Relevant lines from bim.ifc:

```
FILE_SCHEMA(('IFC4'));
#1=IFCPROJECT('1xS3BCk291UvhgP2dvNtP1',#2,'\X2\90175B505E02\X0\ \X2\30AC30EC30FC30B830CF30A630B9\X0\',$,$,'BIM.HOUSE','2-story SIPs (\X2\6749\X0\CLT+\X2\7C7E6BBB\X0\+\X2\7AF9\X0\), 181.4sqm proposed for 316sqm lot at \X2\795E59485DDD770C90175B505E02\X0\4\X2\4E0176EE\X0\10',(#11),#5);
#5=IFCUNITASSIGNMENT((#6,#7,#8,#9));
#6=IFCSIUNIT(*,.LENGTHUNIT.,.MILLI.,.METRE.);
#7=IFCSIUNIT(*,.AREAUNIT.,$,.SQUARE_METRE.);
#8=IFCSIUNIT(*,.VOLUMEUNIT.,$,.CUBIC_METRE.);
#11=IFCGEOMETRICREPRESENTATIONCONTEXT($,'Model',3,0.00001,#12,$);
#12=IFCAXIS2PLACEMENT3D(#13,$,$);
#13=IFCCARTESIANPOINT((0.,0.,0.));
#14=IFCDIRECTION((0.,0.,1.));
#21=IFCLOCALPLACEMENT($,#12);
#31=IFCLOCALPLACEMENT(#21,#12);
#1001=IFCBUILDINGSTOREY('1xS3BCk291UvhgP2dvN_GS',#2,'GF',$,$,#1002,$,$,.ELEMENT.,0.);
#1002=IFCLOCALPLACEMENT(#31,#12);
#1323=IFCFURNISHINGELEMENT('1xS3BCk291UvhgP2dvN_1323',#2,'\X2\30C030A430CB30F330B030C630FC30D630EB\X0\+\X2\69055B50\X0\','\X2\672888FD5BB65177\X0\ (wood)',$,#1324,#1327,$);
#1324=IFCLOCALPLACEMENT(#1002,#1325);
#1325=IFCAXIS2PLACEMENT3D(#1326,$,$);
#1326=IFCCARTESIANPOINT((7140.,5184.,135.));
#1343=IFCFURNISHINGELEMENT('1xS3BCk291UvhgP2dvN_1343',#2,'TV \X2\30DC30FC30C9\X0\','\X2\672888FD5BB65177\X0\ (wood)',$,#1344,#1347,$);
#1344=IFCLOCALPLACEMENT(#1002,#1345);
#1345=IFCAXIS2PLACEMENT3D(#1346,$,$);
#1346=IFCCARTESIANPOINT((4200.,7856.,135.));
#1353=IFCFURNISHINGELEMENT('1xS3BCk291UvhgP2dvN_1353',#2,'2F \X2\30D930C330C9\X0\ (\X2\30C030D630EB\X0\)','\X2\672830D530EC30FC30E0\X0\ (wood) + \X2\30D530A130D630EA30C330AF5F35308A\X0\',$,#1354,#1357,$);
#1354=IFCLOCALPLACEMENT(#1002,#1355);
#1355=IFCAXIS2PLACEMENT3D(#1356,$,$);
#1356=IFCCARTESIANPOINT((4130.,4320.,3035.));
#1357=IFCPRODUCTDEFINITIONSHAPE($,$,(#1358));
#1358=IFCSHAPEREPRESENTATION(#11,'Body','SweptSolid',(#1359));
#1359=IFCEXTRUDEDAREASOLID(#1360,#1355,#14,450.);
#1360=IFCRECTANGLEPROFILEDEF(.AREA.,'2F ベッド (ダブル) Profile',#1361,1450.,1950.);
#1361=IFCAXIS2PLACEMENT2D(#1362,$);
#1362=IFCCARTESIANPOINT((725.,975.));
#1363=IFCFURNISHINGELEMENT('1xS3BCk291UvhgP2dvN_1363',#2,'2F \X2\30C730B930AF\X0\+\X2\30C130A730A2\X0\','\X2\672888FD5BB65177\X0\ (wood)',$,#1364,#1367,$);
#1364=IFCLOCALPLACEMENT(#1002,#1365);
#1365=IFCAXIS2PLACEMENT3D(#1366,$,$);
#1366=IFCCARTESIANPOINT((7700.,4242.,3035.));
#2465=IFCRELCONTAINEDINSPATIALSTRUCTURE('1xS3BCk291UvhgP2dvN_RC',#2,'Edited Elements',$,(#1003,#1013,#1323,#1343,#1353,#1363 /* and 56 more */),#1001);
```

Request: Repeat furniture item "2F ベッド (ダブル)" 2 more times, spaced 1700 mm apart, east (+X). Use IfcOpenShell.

```python
import numpy as np
import ifcopenshell
import ifcopenshell.api.geometry
import ifcopenshell.api.root
import ifcopenshell.util.element
import ifcopenshell.util.placement
import ifcopenshell.util.unit

model = ifcopenshell.open("bim.ifc")
unit_scale = ifcopenshell.util.unit.calculate_unit_scale(model)


def reuse_history(source, copy):
    """copy_class also copies each property set's owner history, people and application; keep the originals."""
    for rel in copy.IsDefinedBy:
        if rel.is_a("IfcRelDefinesByProperties") and (history := rel.RelatingPropertyDefinition.OwnerHistory):
            rel.RelatingPropertyDefinition.OwnerHistory = source.OwnerHistory
            ifcopenshell.util.element.remove_deep2(model, history)


source = model.by_guid("1xS3BCk291UvhgP2dvN_1353")
base = ifcopenshell.util.placement.get_local_placement(source.ObjectPlacement)
step = np.array([1.0, 0.0, 0.0]) * 1.7 / unit_scale

for i in range(1, 3):
    copy = ifcopenshell.api.root.copy_class(model, product=source)
    copy.Representation = ifcopenshell.util.element.copy_deep(
        model, source.Representation, exclude=["IfcGeometricRepresentationContext", "IfcRepresentationMap"]
    )
    reuse_history(source, copy)
    matrix = base.copy()
    matrix[:3, 3] += i * step
    print("added at", matrix[:3, 3].round(3) + 0.0)
    ifcopenshell.api.geometry.edit_object_placement(model, product=copy, matrix=matrix, is_si=False)

model.write("bim_rev.ifc")
```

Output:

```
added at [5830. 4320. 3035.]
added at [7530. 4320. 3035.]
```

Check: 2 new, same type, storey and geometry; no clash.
